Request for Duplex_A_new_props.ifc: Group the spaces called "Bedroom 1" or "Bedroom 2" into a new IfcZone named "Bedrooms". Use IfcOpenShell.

First a look at what the model holds.

```python
import ifcopenshell

model = ifcopenshell.open("Duplex_A_new_props.ifc")
print(model.schema)
seen = {}
for space in model.by_type("IfcSpace"):
    seen[space.LongName] = seen.get(space.LongName, 0) + 1
for name, count in sorted(seen.items(), key=str):
    print(count, "x", name)
print("zones:", [z.Name for z in model.by_type("IfcZone")][:20])
```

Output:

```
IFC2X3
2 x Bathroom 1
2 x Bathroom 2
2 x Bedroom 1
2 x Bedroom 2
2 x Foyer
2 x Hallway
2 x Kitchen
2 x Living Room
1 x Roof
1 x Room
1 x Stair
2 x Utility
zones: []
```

```python
import ifcopenshell
import ifcopenshell.api.group
import ifcopenshell.api.root

model = ifcopenshell.open("Duplex_A_new_props.ifc")

names = {"Bedroom 1", "Bedroom 2"}
spaces = [s for s in model.by_type("IfcSpace") if s.LongName in names]

zone = ifcopenshell.api.root.create_entity(model, ifc_class="IfcZone", name="Bedrooms")
ifcopenshell.api.group.assign_group(model, products=spaces, group=zone)
print(len(spaces), "spaces in", zone.Name)

model.write("Duplex_A_new_props_edited.ifc")
```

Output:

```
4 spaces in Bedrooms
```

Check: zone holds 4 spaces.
